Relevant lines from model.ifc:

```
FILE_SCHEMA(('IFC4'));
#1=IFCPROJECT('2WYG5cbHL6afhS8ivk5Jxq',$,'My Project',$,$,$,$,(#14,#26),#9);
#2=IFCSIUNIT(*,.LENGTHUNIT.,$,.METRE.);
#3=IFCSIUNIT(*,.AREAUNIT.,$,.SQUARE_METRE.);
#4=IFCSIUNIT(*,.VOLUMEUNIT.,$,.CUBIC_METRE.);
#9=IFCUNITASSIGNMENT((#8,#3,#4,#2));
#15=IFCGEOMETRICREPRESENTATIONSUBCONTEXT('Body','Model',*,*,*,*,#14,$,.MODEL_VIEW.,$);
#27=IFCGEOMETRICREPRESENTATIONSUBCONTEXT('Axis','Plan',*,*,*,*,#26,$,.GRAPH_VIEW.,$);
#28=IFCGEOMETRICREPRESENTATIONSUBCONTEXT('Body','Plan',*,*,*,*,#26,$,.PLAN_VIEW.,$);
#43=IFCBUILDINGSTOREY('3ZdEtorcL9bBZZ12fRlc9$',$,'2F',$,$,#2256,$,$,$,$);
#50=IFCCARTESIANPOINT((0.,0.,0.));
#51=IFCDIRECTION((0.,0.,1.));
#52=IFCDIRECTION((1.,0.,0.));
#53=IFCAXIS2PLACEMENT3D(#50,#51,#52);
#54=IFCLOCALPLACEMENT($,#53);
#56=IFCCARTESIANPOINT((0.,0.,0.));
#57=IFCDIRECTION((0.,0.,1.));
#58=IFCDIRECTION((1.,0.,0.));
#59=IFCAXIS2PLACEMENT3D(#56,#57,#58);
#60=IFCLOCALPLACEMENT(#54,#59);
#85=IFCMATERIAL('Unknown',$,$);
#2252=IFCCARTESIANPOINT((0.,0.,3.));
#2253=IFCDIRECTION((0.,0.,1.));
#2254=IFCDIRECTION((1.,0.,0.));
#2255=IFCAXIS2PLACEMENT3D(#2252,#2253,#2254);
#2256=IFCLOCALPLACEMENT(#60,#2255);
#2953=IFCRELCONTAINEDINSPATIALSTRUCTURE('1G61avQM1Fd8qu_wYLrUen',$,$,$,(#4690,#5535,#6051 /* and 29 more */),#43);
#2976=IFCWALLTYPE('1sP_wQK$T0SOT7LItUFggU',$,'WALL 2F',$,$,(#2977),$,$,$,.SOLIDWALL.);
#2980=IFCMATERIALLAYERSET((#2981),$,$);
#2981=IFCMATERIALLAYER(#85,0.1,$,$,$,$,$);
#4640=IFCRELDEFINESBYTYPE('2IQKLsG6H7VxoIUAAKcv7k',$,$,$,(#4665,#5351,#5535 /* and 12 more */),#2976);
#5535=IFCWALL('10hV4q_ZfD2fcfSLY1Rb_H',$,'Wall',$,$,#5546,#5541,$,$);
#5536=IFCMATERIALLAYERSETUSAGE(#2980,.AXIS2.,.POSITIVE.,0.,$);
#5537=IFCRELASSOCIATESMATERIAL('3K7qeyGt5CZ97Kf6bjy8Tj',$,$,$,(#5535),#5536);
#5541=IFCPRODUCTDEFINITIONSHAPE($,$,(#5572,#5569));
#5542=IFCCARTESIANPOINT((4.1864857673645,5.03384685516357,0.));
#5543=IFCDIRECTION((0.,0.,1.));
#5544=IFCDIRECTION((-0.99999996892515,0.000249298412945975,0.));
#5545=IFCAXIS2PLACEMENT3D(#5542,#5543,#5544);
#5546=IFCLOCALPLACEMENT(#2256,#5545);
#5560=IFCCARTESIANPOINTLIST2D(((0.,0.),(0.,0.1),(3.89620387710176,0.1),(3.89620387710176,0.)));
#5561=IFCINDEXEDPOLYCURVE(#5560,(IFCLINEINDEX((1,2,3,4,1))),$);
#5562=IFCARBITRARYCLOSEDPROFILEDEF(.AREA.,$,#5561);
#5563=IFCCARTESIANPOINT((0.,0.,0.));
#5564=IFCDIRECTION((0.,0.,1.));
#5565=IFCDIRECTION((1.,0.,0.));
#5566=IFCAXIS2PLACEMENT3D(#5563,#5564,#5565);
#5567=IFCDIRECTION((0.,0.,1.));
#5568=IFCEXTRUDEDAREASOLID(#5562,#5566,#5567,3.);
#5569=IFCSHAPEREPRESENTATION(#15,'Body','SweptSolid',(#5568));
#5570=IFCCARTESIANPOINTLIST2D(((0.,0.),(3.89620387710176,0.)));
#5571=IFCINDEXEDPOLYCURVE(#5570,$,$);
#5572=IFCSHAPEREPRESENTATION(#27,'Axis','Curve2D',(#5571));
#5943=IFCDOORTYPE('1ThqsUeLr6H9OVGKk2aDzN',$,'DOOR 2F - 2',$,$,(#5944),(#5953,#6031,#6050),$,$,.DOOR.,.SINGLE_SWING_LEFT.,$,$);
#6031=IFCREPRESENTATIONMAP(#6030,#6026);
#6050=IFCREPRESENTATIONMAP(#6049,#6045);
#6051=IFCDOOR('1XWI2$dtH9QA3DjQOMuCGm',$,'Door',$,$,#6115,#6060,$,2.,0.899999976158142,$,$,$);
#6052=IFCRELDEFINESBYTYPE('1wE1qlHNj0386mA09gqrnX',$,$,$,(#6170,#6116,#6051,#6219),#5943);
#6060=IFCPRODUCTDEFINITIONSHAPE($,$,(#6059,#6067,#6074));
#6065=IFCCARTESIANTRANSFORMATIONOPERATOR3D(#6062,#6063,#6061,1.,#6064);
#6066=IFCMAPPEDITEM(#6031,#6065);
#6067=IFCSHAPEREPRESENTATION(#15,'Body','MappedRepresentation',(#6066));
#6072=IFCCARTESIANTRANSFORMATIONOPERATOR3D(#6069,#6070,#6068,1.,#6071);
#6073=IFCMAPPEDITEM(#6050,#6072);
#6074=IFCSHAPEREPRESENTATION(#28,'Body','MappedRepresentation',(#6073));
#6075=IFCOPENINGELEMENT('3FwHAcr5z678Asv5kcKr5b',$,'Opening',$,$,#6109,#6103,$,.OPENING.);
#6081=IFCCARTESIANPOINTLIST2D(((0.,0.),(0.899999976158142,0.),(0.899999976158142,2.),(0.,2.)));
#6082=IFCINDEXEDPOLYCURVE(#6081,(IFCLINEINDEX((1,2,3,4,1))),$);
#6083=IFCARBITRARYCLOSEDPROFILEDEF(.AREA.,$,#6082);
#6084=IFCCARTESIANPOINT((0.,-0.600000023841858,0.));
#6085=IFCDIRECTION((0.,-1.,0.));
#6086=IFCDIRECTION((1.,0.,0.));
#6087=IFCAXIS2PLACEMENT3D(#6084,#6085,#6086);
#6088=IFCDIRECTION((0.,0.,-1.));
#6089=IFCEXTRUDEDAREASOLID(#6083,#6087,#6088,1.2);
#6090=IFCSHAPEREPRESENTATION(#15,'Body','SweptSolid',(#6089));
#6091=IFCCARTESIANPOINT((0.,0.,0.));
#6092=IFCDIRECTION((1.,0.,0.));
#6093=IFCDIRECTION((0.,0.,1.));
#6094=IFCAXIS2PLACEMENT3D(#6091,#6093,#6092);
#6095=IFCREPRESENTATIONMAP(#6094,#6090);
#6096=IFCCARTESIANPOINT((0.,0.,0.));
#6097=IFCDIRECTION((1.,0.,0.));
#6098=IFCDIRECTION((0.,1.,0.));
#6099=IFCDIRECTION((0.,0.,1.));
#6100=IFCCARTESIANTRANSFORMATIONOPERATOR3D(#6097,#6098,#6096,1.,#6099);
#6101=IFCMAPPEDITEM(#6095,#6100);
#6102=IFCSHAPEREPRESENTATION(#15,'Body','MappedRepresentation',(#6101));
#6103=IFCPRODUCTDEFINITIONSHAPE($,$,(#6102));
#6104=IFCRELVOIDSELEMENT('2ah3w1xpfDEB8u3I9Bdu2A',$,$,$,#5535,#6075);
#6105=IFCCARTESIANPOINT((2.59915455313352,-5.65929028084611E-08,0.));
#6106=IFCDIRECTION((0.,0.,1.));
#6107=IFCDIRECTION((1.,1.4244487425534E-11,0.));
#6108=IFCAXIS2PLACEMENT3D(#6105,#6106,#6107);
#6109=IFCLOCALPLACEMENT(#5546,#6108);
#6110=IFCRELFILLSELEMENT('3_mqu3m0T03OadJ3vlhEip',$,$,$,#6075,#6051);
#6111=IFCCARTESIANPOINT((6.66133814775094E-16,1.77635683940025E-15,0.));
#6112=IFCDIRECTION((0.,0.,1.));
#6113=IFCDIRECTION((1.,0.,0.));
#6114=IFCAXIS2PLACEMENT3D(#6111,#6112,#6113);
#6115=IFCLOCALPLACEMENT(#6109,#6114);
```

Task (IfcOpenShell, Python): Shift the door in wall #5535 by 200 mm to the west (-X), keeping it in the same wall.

```python
import ifcopenshell
import ifcopenshell.api.geometry
import ifcopenshell.util.placement
import ifcopenshell.util.unit

model = ifcopenshell.open("model.ifc")
unit_scale = ifcopenshell.util.unit.calculate_unit_scale(model)

door = model.by_id(6051)
opening = door.FillsVoids[0].RelatingOpeningElement
wall = opening.VoidsElements[0].RelatingBuildingElement

wall_matrix = ifcopenshell.util.placement.get_local_placement(wall.ObjectPlacement)
shift = wall_matrix[:3, 0] * 0.2 / unit_scale
before = ifcopenshell.util.placement.get_local_placement(door.ObjectPlacement)[:3, 3].copy()

# The door is placed relative to its opening, so it follows when the opening moves.
matrix = ifcopenshell.util.placement.get_local_placement(opening.ObjectPlacement)
matrix[:3, 3] += shift
ifcopenshell.api.geometry.edit_object_placement(
    model, product=opening, matrix=matrix, is_si=False, should_transform_children=True
)

after = ifcopenshell.util.placement.get_local_placement(door.ObjectPlacement)[:3, 3]
print("door moved by", (after - before).round(3) + 0.0)

model.write("model_rev.ifc")
```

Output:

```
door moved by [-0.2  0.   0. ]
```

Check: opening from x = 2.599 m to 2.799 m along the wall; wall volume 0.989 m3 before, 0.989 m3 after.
